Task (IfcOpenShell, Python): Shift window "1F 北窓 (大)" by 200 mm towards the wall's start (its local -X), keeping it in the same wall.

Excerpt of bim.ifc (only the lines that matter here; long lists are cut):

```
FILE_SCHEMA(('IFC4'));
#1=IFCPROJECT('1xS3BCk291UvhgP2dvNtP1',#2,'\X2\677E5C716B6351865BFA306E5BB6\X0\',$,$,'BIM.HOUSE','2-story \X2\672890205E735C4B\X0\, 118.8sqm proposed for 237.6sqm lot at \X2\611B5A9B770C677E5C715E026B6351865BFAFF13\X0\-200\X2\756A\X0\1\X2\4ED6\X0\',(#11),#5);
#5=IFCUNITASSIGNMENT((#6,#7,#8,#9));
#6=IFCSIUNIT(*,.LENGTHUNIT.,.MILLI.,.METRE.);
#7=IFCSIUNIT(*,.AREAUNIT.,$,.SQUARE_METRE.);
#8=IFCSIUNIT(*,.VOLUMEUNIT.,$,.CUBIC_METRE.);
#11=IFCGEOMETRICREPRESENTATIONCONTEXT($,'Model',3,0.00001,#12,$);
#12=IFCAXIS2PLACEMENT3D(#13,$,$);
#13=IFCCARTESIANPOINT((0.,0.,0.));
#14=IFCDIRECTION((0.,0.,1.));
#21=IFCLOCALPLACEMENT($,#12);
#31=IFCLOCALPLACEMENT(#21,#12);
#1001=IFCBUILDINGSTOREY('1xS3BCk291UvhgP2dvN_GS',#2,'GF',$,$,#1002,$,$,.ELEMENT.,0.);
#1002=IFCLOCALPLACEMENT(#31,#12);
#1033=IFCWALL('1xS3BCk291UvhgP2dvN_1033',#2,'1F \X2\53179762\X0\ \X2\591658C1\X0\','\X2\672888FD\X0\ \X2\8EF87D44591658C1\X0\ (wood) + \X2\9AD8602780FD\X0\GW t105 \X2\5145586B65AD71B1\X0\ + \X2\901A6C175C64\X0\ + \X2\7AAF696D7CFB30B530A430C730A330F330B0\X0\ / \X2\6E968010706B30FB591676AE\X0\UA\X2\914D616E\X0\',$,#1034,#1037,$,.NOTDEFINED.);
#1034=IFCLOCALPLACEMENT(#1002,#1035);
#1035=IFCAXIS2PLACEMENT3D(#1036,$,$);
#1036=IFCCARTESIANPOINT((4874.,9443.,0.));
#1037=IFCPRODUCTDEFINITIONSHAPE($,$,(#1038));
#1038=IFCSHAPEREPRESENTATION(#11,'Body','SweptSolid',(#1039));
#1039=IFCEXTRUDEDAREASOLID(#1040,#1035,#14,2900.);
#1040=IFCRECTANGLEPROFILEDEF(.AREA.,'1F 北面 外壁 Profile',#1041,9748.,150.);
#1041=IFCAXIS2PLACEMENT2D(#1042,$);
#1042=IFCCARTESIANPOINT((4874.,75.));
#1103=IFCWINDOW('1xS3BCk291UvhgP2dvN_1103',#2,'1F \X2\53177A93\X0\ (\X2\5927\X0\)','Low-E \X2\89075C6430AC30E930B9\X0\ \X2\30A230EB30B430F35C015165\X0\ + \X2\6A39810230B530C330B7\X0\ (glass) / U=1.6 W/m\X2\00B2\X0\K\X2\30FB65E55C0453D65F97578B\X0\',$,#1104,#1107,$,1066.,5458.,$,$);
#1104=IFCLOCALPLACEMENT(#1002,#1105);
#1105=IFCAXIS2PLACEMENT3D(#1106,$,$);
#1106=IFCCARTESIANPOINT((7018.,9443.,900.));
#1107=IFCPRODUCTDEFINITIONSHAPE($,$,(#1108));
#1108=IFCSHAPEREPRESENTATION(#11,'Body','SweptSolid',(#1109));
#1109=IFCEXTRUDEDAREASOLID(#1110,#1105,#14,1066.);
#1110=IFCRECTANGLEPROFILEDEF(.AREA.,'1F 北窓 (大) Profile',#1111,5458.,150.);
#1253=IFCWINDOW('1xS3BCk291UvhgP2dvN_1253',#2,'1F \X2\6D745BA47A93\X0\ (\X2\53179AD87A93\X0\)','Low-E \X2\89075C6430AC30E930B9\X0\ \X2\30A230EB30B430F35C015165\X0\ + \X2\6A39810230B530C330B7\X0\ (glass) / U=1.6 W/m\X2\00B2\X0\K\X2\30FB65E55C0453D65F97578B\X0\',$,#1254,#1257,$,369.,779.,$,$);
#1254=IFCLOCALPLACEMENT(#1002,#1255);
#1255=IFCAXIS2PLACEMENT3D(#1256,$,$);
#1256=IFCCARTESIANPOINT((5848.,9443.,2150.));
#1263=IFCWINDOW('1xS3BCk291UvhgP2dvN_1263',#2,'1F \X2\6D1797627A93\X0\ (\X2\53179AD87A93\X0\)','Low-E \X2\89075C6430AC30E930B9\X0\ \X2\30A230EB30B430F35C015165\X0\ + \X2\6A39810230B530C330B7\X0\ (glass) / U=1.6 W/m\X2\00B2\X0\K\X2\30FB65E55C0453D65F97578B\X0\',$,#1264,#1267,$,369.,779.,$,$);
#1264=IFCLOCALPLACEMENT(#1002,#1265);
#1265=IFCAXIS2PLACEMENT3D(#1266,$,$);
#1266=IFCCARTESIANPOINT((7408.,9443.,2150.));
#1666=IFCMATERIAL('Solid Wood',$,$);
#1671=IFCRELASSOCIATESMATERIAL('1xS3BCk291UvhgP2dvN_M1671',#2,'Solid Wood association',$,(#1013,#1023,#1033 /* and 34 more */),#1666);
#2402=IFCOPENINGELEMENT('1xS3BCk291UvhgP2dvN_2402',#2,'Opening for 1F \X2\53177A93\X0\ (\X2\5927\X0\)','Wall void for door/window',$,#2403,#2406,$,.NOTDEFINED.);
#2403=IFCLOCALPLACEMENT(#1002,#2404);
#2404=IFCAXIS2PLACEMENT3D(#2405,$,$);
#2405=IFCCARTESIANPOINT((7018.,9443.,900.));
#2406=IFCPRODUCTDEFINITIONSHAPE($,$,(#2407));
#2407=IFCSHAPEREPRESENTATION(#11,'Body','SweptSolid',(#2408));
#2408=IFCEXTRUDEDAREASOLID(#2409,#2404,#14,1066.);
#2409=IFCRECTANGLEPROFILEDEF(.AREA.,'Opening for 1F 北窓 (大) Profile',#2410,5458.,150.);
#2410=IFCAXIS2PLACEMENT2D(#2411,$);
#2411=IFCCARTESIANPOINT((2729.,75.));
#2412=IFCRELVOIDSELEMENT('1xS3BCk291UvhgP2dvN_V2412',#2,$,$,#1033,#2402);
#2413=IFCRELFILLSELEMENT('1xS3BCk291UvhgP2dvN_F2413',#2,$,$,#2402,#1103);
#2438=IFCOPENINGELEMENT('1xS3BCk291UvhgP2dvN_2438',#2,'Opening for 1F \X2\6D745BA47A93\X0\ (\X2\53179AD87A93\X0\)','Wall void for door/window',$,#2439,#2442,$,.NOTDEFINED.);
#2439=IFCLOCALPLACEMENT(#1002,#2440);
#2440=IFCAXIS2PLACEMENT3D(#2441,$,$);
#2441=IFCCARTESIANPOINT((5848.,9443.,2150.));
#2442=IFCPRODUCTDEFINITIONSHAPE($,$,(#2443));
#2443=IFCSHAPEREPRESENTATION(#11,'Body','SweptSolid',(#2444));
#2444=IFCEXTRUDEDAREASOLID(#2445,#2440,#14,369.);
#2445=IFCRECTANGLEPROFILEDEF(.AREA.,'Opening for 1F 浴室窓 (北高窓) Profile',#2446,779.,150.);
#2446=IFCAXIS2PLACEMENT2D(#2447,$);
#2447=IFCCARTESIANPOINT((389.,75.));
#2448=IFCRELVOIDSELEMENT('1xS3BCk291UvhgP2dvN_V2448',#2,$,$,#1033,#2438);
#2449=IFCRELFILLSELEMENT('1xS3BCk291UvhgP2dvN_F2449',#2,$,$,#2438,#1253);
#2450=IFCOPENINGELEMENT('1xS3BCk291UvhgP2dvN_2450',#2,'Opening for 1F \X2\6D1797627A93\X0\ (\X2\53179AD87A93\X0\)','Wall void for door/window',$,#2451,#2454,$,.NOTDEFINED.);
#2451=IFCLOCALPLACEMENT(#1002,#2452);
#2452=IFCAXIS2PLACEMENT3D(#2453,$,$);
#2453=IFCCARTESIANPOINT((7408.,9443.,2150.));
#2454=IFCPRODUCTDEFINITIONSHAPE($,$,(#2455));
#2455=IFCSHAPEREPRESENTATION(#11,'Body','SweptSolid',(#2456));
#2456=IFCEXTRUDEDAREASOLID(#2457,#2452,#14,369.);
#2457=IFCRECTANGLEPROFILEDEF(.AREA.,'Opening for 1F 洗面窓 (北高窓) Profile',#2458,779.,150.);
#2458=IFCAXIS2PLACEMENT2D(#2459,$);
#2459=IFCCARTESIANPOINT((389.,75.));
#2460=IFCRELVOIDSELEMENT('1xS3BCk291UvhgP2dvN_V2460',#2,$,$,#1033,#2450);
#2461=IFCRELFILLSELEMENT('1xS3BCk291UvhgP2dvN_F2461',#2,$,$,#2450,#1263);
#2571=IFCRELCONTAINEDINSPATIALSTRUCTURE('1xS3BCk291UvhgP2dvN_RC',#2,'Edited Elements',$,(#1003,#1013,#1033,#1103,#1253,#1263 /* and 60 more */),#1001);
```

```python
import ifcopenshell
import ifcopenshell.api.geometry
import ifcopenshell.util.placement
import ifcopenshell.util.unit

model = ifcopenshell.open("bim.ifc")
unit_scale = ifcopenshell.util.unit.calculate_unit_scale(model)

window = model.by_id(1103)
opening = window.FillsVoids[0].RelatingOpeningElement
wall = opening.VoidsElements[0].RelatingBuildingElement

wall_matrix = ifcopenshell.util.placement.get_local_placement(wall.ObjectPlacement)
shift = wall_matrix[:3, 0] * -0.2 / unit_scale
before = ifcopenshell.util.placement.get_local_placement(window.ObjectPlacement)[:3, 3].copy()

# The window is not placed relative to its opening, so move both.
for product in (opening, window):
    matrix = ifcopenshell.util.placement.get_local_placement(product.ObjectPlacement)
    matrix[:3, 3] += shift
    ifcopenshell.api.geometry.edit_object_placement(model, product=product, matrix=matrix, is_si=False)

after = ifcopenshell.util.placement.get_local_placement(window.ObjectPlacement)[:3, 3]
print("window moved by", (after - before).round(3) + 0.0)

model.write("bim-out.ifc")
```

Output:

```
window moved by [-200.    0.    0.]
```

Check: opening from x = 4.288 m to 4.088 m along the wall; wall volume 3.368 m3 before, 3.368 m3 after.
